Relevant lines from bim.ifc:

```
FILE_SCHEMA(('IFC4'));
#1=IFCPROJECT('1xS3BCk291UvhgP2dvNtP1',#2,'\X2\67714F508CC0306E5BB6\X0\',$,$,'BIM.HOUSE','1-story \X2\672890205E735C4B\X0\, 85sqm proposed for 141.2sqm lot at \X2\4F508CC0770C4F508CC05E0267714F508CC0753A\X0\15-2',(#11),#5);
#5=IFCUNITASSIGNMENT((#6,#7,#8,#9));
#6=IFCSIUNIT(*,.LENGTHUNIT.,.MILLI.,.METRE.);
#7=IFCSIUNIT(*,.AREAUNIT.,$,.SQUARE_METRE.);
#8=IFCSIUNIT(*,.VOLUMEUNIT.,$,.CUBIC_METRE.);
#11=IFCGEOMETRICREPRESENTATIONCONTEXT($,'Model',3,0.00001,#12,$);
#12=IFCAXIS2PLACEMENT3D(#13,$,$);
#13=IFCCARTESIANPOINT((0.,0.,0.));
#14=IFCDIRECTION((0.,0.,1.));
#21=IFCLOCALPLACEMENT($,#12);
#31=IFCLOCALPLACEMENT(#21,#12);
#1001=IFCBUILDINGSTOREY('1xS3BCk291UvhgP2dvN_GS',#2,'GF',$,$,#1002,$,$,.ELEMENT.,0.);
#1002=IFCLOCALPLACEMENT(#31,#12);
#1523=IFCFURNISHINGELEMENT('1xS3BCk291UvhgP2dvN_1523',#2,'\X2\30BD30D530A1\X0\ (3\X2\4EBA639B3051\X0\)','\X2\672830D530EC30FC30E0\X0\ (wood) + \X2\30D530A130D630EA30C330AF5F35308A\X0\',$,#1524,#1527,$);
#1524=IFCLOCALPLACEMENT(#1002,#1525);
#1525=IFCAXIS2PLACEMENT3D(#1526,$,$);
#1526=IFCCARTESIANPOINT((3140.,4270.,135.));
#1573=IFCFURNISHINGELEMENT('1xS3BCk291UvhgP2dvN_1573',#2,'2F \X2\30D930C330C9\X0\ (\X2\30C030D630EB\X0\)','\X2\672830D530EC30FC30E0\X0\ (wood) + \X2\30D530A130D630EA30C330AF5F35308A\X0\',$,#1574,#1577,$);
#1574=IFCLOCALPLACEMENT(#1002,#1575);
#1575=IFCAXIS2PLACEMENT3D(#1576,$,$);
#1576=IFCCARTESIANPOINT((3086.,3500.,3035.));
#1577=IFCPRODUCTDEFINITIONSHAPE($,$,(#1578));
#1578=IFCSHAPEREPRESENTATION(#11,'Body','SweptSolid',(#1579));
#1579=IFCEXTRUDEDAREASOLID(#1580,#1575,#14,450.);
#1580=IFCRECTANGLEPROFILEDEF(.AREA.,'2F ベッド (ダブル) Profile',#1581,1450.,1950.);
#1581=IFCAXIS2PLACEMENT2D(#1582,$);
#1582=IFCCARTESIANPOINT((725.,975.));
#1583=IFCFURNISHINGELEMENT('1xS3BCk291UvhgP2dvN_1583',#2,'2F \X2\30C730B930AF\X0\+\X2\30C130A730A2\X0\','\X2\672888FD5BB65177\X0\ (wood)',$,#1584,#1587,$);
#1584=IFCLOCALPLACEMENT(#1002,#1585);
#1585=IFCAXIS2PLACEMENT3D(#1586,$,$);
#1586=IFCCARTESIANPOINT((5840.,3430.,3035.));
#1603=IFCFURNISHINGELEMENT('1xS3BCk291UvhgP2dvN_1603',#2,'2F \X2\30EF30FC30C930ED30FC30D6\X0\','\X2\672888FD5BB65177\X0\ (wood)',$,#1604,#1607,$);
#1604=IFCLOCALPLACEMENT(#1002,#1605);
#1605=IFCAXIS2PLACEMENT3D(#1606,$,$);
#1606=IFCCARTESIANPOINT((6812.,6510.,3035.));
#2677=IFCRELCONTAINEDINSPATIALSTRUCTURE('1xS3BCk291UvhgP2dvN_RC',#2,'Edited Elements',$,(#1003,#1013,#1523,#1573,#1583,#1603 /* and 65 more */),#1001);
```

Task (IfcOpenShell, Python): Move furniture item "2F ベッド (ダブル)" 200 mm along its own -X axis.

```python
import ifcopenshell
import ifcopenshell.api.geometry
import ifcopenshell.util.placement
import ifcopenshell.util.unit

model = ifcopenshell.open("bim.ifc")
unit_scale = ifcopenshell.util.unit.calculate_unit_scale(model)

item = model.by_guid("1xS3BCk291UvhgP2dvN_1573")
matrix = ifcopenshell.util.placement.get_local_placement(item.ObjectPlacement)
matrix[:3, 3] -= matrix[:3, 0] * 0.2 / unit_scale
ifcopenshell.api.geometry.edit_object_placement(model, product=item, matrix=matrix, is_si=False)

print(ifcopenshell.util.placement.get_local_placement(item.ObjectPlacement).round(3) + 0.0)

model.write("bim_edited.ifc")
```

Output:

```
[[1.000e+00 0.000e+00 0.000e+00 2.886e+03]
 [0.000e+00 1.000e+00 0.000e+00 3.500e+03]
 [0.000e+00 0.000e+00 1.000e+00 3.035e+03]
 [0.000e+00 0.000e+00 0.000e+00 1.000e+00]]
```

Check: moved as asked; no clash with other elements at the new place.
